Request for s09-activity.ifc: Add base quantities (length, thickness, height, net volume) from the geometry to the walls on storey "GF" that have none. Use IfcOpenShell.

First a look at what the model holds.

```python
import ifcopenshell
import ifcopenshell.util.element
import ifcopenshell.util.unit

model = ifcopenshell.open("s09-activity.ifc")
print(model.schema)
for unit_type in ("LENGTHUNIT", "AREAUNIT", "VOLUMEUNIT"):
    print(unit_type, ifcopenshell.util.unit.calculate_unit_scale(model, unit_type))
storey = next(s for s in model.by_type("IfcBuildingStorey") if s.Name == "GF")
walls = [e for e in ifcopenshell.util.element.get_decomposition(storey) if e.is_a("IfcWall")]
for e in sorted(walls, key=lambda e: e.id()):
    print(e.id(), e.is_a(), e.Name, list(ifcopenshell.util.element.get_psets(e, qtos_only=True)), sep=" | ")
```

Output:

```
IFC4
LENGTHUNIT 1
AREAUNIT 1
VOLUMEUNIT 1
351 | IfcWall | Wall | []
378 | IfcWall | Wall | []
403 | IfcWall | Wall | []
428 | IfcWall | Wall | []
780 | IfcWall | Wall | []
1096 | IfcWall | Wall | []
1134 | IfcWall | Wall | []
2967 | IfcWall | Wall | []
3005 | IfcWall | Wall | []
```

```python
import ifcopenshell
import ifcopenshell.api.pset
import ifcopenshell.geom
import ifcopenshell.util.element
import ifcopenshell.util.shape
import ifcopenshell.util.unit

model = ifcopenshell.open("s09-activity.ifc")
unit_scale = ifcopenshell.util.unit.calculate_unit_scale(model)
volume_scale = ifcopenshell.util.unit.calculate_unit_scale(model, "VOLUMEUNIT")
settings = ifcopenshell.geom.settings()

storey = next(s for s in model.by_type("IfcBuildingStorey") if s.Name == "GF")
walls = [e for e in ifcopenshell.util.element.get_decomposition(storey) if e.is_a("IfcWall")]

for e in sorted(walls, key=lambda e: e.id()):
    if ifcopenshell.util.element.get_psets(e, qtos_only=True, should_inherit=False):
        continue
    # Geometry comes back in metres, in the element's own axes.
    shape = ifcopenshell.geom.create_shape(settings, e)
    values = {
        "Length": ifcopenshell.util.shape.get_x(shape.geometry) / unit_scale,
        "Width": ifcopenshell.util.shape.get_y(shape.geometry) / unit_scale,
        "Height": ifcopenshell.util.shape.get_z(shape.geometry) / unit_scale,
        "NetVolume": ifcopenshell.util.shape.get_volume(shape.geometry) / volume_scale,
    }
    qto = ifcopenshell.api.pset.add_qto(model, product=e, name="Qto_WallBaseQuantities")
    ifcopenshell.api.pset.edit_qto(model, qto=qto, properties=values)
    print(e.id(), {k: round(v, 3) for k, v in values.items()})

model.write("s09-activity_updated.ifc")
```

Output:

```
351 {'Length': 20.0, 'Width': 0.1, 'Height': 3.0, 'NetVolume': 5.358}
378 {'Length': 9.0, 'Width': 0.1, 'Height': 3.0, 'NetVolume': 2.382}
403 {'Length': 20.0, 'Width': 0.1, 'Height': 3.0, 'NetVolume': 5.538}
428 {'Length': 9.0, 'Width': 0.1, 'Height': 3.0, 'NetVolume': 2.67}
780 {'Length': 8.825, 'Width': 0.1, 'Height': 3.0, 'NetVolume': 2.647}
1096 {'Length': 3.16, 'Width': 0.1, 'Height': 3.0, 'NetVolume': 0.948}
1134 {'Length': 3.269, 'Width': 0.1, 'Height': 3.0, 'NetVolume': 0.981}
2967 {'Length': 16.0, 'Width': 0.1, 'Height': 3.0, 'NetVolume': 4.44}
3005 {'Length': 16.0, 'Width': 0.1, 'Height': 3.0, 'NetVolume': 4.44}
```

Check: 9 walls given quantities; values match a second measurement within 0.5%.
